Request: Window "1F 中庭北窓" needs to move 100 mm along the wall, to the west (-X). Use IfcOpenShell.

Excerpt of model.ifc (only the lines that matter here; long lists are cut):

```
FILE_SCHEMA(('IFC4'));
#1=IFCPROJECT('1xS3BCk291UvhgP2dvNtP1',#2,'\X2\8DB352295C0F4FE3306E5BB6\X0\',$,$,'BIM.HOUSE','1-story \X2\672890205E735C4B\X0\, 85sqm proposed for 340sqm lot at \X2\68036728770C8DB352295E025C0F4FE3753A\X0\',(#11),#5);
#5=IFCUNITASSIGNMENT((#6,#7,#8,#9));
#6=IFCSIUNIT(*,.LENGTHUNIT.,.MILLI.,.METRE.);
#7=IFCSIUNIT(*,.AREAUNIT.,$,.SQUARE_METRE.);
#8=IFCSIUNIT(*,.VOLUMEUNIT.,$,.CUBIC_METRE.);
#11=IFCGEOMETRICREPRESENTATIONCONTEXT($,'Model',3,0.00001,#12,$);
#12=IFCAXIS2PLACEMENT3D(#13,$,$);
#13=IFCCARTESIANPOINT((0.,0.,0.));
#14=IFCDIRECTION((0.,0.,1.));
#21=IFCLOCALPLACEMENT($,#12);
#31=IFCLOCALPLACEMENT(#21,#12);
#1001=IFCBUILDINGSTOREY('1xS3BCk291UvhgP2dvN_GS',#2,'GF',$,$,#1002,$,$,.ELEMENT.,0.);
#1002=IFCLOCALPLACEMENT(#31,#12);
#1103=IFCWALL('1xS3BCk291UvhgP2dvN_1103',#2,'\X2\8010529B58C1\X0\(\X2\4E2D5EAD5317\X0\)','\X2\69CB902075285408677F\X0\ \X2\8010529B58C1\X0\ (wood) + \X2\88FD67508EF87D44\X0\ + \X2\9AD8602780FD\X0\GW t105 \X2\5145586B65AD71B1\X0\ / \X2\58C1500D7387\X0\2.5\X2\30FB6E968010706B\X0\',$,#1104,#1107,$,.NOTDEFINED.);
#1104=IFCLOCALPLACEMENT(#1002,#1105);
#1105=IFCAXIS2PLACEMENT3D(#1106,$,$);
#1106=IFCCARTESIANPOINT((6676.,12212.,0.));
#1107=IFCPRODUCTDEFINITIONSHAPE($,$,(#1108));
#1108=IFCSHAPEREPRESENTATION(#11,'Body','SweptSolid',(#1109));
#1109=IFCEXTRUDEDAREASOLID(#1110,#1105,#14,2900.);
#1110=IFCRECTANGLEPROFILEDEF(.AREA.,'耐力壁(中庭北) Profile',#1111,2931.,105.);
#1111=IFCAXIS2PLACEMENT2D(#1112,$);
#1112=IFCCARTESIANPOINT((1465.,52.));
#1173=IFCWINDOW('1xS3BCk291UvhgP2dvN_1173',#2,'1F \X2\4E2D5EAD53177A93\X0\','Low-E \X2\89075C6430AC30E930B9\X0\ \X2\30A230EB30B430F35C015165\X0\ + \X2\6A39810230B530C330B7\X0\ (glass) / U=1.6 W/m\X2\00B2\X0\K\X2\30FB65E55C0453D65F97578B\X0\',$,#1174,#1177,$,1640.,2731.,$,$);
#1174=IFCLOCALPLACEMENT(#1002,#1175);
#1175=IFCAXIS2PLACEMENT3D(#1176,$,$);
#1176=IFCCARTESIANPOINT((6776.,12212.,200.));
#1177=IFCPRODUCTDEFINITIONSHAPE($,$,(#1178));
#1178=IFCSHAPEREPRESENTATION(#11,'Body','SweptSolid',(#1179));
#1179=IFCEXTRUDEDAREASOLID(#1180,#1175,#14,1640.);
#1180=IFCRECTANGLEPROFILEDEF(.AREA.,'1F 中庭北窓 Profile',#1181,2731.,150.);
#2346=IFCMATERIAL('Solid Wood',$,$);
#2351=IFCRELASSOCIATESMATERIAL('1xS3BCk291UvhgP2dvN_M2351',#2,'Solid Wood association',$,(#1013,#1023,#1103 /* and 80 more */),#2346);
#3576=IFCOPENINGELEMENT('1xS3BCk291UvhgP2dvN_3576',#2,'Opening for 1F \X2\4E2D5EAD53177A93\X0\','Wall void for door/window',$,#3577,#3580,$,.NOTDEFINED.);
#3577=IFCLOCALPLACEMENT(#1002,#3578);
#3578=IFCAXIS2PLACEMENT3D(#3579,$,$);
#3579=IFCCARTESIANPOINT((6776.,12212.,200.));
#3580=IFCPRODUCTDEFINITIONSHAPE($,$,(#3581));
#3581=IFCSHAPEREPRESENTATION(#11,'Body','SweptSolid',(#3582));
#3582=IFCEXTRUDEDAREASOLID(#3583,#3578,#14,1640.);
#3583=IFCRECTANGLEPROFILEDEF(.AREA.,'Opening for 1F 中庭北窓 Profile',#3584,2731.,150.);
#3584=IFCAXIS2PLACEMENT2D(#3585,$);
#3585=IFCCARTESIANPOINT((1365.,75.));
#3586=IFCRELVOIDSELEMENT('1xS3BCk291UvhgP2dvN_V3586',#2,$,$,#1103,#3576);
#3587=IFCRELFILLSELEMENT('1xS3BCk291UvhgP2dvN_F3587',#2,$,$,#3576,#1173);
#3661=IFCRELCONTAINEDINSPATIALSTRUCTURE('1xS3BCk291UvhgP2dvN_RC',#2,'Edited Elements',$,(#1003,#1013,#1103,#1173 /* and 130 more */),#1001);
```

```python
import ifcopenshell
import ifcopenshell.api.geometry
import ifcopenshell.util.placement
import ifcopenshell.util.unit

model = ifcopenshell.open("model.ifc")
unit_scale = ifcopenshell.util.unit.calculate_unit_scale(model)

window = model.by_guid("1xS3BCk291UvhgP2dvN_1173")
opening = window.FillsVoids[0].RelatingOpeningElement
wall = opening.VoidsElements[0].RelatingBuildingElement

wall_matrix = ifcopenshell.util.placement.get_local_placement(wall.ObjectPlacement)
shift = wall_matrix[:3, 0] * -0.1 / unit_scale
before = ifcopenshell.util.placement.get_local_placement(window.ObjectPlacement)[:3, 3].copy()

# The window is not placed relative to its opening, so move both.
for product in (opening, window):
    matrix = ifcopenshell.util.placement.get_local_placement(product.ObjectPlacement)
    matrix[:3, 3] += shift
    ifcopenshell.api.geometry.edit_object_placement(model, product=product, matrix=matrix, is_si=False)

after = ifcopenshell.util.placement.get_local_placement(window.ObjectPlacement)[:3, 3]
print("window moved by", (after - before).round(3) + 0.0)

model.write("model_updated.ifc")
```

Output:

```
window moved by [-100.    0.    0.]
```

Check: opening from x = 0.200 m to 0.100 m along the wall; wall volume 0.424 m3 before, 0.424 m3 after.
